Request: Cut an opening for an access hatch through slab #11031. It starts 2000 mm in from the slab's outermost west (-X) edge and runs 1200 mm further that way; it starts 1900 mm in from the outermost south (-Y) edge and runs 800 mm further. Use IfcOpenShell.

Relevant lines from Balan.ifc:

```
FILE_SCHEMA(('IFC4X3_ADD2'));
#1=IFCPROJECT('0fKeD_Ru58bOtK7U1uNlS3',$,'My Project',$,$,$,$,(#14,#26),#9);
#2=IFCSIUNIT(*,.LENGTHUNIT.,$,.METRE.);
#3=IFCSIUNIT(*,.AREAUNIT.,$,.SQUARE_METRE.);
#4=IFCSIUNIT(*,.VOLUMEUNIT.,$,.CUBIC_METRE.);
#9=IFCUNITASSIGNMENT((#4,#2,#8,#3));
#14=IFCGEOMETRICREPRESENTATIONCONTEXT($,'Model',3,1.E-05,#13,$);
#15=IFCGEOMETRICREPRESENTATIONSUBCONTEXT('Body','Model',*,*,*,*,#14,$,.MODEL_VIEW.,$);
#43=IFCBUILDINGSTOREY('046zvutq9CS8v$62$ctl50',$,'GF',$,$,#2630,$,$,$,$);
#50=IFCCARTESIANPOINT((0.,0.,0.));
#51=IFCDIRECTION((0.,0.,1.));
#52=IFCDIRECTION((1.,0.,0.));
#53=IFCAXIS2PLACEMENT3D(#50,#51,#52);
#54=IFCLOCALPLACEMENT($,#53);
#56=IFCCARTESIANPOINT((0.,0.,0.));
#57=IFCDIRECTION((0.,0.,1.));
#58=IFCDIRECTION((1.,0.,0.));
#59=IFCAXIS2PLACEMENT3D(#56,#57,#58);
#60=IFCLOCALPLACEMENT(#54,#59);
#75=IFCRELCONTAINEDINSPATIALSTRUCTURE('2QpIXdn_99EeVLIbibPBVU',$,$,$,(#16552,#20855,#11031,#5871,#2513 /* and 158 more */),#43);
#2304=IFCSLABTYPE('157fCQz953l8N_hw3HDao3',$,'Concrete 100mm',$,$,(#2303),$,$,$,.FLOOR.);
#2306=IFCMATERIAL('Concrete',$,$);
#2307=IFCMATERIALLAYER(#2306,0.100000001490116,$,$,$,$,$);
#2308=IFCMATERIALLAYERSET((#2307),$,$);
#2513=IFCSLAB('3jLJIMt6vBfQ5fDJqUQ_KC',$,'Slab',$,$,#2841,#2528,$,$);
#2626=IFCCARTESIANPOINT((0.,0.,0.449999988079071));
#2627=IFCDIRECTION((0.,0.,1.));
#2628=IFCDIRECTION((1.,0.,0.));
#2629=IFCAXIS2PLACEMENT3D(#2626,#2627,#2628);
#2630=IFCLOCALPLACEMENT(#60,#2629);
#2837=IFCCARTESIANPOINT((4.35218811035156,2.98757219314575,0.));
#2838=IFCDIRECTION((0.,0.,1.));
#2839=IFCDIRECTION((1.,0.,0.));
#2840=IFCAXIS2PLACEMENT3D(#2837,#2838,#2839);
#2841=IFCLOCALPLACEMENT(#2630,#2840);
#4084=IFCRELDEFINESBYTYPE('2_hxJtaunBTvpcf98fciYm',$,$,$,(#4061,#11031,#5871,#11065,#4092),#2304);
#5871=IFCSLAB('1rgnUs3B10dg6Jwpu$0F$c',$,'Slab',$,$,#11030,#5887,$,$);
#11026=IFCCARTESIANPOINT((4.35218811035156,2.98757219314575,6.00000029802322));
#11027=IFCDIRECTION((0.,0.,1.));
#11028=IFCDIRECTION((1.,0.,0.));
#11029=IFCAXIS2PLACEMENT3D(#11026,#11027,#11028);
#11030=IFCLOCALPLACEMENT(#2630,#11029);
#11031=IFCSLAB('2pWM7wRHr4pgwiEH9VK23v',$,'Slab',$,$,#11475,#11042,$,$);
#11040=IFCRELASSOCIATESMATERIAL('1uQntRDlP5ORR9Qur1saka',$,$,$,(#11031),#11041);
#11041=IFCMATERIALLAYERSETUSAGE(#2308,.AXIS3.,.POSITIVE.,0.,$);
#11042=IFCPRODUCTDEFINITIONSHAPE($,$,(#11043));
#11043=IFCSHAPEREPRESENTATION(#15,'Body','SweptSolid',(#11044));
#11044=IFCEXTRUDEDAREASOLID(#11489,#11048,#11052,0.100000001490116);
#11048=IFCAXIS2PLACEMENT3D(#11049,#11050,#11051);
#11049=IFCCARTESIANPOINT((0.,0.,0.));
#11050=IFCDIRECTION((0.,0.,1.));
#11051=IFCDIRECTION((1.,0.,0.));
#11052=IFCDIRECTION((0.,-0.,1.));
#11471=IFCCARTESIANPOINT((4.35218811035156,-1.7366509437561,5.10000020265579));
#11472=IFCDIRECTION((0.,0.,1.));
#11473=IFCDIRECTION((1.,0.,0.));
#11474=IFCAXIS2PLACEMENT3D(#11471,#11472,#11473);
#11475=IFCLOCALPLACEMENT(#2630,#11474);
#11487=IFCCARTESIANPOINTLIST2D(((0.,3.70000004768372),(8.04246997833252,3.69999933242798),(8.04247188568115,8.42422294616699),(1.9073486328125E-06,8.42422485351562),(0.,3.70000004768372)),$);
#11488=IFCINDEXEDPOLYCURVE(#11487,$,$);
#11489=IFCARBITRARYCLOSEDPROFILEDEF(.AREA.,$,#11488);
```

```python
import numpy as np
import ifcopenshell
import ifcopenshell.api.feature
import ifcopenshell.api.geometry
import ifcopenshell.api.root
import ifcopenshell.geom
import ifcopenshell.util.placement
import ifcopenshell.util.representation
import ifcopenshell.util.shape
import ifcopenshell.util.unit

model = ifcopenshell.open("Balan.ifc")
unit_scale = ifcopenshell.util.unit.calculate_unit_scale(model)
settings = ifcopenshell.geom.settings()


def volume(element):
    """Net volume in cubic metres, openings subtracted."""
    shape = ifcopenshell.geom.create_shape(settings, element)
    return ifcopenshell.util.shape.get_volume(shape.geometry)


slab = model.by_id(11031)
before = volume(slab)

# Extent in the slab's own axes, in metres. The edges named are its -X and -Y sides.
slab_shape = ifcopenshell.geom.create_shape(settings, slab)
vertices = ifcopenshell.util.shape.get_vertices(slab_shape.geometry)
x_min, y_min, bottom = vertices.min(axis=0)
top = vertices[:, 2].max()

opening = ifcopenshell.api.root.create_entity(model, ifc_class="IfcOpeningElement", name="Access hatch opening", predefined_type="OPENING")
context = ifcopenshell.util.representation.get_context(model, "Model", "Body", "MODEL_VIEW")
width, depth = 1.2, 0.8
outline = [(0.0, 0.0), (width, 0.0), (width, depth), (0.0, depth), (0.0, 0.0)]
# Overshoot both faces by 50 mm so the cut is clean.
shape = ifcopenshell.api.geometry.add_slab_representation(
    model, context=context, depth=top - bottom + 0.1, polyline=outline
)
ifcopenshell.api.geometry.assign_representation(model, product=opening, representation=shape)

matrix = ifcopenshell.util.placement.get_local_placement(slab.ObjectPlacement)
matrix[:, 3] = matrix @ np.append(np.array([x_min + 2, y_min + 1.9, bottom - 0.05]) / unit_scale, 1.0)
ifcopenshell.api.geometry.edit_object_placement(model, product=opening, matrix=matrix, is_si=False)
ifcopenshell.api.feature.add_feature(model, feature=opening, element=slab)

after = volume(slab)

print(f"slab volume {before:.3f} -> {after:.3f} m3")

model.write("Balan_edited.ifc")
```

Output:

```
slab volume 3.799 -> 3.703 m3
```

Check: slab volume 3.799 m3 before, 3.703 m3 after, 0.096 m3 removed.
